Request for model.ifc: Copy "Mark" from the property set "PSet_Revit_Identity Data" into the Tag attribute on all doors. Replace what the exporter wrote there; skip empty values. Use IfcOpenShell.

First a look at what the model holds.

```python
import ifcopenshell
import ifcopenshell.util.element

model = ifcopenshell.open("model.ifc")
print(model.schema)
doors = model.by_type("IfcDoor")
print(len(doors), "doors")
for e in doors[:8]:
    source = ifcopenshell.util.element.get_pset(e, "PSet_Revit_Identity Data", "Mark")
    target = e.Tag
    print(e.id(), repr(source), repr(target), sep=" | ")
```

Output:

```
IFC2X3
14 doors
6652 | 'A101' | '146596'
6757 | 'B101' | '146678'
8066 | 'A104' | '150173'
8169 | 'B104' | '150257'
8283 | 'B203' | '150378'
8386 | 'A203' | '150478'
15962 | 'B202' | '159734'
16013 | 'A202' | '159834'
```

```python
import ifcopenshell
import ifcopenshell.util.element

model = ifcopenshell.open("model.ifc")

count = 0
for e in model.by_type("IfcDoor"):
    value = ifcopenshell.util.element.get_pset(e, "PSet_Revit_Identity Data", "Mark")
    current = e.Tag
    if not value or not value.strip() or current == value:
        continue
    e.Tag = value
    count += 1

print(count, "doors updated")

model.write("model_edited.ifc")
```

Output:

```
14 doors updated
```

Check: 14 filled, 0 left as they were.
